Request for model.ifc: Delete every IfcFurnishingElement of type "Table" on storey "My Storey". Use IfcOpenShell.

First a look at what the model holds.

```python
import ifcopenshell
import ifcopenshell.util.element

model = ifcopenshell.open("model.ifc")
print(model.schema)
storey = next(s for s in model.by_type("IfcBuildingStorey") if s.Name == "My Storey")
furniture = [e for e in ifcopenshell.util.element.get_decomposition(storey) if e.is_a("IfcFurnishingElement")]
seen = {}
for e in furniture:
    element_type = ifcopenshell.util.element.get_type(e)
    name = element_type.Name if element_type not in (None, e) else None
    seen[name] = seen.get(name, 0) + 1
for name, count in sorted(seen.items(), key=str):
    print(count, "x", name)
```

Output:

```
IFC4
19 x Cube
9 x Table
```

```python
import ifcopenshell
import ifcopenshell.api.root
import ifcopenshell.util.element

model = ifcopenshell.open("model.ifc")

storey = next(s for s in model.by_type("IfcBuildingStorey") if s.Name == "My Storey")
furniture = [e for e in ifcopenshell.util.element.get_decomposition(storey) if e.is_a("IfcFurnishingElement")]
targets = [e for e in furniture if (t := ifcopenshell.util.element.get_type(e)) not in (None, e) and t.Name == "Table"]

for e in targets:
    ifcopenshell.api.root.remove_product(model, product=e)
print(len(targets), "removed")

model.write("model-out.ifc")
```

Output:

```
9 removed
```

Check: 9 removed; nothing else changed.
